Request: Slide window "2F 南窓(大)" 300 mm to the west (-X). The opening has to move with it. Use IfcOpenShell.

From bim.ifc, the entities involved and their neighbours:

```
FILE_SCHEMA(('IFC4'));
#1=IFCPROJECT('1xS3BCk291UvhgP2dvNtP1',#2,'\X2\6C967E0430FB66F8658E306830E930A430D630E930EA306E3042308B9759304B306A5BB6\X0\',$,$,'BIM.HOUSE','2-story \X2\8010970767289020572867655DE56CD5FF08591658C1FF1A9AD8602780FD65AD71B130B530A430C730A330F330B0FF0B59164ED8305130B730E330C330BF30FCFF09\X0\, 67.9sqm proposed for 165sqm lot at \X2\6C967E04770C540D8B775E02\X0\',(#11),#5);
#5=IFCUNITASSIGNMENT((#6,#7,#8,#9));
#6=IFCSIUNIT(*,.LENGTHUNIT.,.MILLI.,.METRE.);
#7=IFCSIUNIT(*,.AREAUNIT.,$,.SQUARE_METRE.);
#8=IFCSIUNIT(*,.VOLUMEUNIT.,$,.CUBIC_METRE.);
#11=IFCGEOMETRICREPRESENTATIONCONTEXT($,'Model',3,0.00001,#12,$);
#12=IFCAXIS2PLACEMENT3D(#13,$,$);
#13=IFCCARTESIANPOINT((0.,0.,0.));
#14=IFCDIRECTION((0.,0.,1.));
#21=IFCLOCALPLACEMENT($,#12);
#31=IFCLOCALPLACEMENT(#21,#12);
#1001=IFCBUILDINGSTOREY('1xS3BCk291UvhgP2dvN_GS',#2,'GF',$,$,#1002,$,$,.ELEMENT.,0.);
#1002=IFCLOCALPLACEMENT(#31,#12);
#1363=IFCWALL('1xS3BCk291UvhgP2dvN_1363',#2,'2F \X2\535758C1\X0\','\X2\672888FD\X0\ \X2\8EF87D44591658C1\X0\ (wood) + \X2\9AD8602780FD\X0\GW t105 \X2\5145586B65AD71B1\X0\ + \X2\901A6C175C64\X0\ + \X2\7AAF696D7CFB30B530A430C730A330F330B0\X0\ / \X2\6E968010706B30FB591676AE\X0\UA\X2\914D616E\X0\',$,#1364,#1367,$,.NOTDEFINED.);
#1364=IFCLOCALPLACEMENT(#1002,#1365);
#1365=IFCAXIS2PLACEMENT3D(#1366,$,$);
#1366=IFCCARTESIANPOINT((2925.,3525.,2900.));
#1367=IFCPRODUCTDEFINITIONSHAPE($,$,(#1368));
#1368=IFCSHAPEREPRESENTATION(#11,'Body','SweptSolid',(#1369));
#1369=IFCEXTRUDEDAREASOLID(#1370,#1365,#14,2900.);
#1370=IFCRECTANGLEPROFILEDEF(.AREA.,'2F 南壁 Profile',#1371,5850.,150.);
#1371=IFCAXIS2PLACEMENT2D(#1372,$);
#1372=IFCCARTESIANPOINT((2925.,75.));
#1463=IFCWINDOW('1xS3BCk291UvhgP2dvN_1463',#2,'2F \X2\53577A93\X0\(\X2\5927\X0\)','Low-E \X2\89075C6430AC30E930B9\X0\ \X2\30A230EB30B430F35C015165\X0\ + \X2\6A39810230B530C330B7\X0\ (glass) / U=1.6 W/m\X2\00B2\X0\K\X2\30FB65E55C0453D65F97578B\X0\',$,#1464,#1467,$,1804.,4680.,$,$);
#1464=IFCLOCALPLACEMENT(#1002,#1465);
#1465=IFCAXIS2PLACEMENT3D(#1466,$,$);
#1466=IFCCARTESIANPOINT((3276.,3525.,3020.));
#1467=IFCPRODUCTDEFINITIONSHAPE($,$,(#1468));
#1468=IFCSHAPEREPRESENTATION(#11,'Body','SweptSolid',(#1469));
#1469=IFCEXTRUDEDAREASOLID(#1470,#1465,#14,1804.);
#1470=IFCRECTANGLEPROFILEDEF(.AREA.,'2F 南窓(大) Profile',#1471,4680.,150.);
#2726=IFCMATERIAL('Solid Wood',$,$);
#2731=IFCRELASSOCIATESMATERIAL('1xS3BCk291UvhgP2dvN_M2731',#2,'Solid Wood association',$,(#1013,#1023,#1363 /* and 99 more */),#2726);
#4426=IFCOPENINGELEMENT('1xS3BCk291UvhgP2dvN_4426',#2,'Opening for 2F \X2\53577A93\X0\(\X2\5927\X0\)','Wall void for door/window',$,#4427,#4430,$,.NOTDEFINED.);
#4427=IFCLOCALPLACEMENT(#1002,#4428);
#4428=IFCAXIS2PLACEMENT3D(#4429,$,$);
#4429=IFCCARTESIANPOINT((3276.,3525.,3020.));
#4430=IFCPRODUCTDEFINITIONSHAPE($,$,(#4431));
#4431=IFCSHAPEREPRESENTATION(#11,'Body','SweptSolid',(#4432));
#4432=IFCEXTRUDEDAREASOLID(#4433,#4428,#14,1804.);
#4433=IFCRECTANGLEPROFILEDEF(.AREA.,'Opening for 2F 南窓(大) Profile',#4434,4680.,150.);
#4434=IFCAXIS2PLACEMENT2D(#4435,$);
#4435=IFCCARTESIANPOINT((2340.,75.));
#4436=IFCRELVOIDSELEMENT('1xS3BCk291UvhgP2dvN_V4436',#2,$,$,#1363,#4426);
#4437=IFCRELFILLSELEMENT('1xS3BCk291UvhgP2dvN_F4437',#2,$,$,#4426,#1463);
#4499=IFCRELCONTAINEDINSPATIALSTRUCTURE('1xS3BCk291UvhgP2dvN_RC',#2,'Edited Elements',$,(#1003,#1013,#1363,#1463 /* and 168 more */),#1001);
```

```python
import ifcopenshell
import ifcopenshell.api.geometry
import ifcopenshell.util.placement
import ifcopenshell.util.unit

model = ifcopenshell.open("bim.ifc")
unit_scale = ifcopenshell.util.unit.calculate_unit_scale(model)

window = model.by_guid("1xS3BCk291UvhgP2dvN_1463")
opening = window.FillsVoids[0].RelatingOpeningElement
wall = opening.VoidsElements[0].RelatingBuildingElement

wall_matrix = ifcopenshell.util.placement.get_local_placement(wall.ObjectPlacement)
shift = wall_matrix[:3, 0] * -0.3 / unit_scale
before = ifcopenshell.util.placement.get_local_placement(window.ObjectPlacement)[:3, 3].copy()

# The window is not placed relative to its opening, so move both.
for product in (opening, window):
    matrix = ifcopenshell.util.placement.get_local_placement(product.ObjectPlacement)
    matrix[:3, 3] += shift
    ifcopenshell.api.geometry.edit_object_placement(model, product=product, matrix=matrix, is_si=False)

after = ifcopenshell.util.placement.get_local_placement(window.ObjectPlacement)[:3, 3]
print("window moved by", (after - before).round(3) + 0.0)

model.write("bim-out.ifc")
```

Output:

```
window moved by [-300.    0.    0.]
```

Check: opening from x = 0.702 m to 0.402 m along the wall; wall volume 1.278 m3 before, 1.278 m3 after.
